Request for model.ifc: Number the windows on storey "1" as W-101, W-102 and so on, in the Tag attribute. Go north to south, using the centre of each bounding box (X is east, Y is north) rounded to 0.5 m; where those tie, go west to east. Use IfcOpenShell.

First a look at what the model holds.

```python
import ifcopenshell
import ifcopenshell.util.element
import ifcopenshell.util.placement

model = ifcopenshell.open("model.ifc")
print(model.schema)
storey = next(s for s in model.by_type("IfcBuildingStorey") if s.Name == "1")
windows = [e for e in ifcopenshell.util.element.get_decomposition(storey) if e.is_a("IfcWindow")]
for e in sorted(windows, key=lambda e: e.id()):
    origin = ifcopenshell.util.placement.get_local_placement(e.ObjectPlacement)[:3, 3]
    print(e.id(), e.Tag, e.Name, origin.round(2) + 0.0, sep=" | ")
```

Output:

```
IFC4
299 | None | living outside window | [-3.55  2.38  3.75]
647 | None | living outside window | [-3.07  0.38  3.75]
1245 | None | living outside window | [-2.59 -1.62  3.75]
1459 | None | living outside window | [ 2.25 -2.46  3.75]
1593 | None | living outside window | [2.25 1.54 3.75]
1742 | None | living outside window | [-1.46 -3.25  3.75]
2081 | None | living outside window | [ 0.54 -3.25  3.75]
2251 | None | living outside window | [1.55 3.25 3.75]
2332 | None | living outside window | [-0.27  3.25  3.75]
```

```python
import ifcopenshell
import ifcopenshell.geom
import ifcopenshell.util.element
import ifcopenshell.util.shape

model = ifcopenshell.open("model.ifc")
settings = ifcopenshell.geom.settings()
settings.set("use-world-coords", True)


def centre(element):
    shape = ifcopenshell.geom.create_shape(settings, element)
    return ifcopenshell.util.shape.get_bbox_centroid(shape.geometry)


storey = next(s for s in model.by_type("IfcBuildingStorey") if s.Name == "1")
windows = [e for e in ifcopenshell.util.element.get_decomposition(storey) if e.is_a("IfcWindow")]

# Insertion points can sit at a corner or the storey origin, so sort by the geometry (in metres).
centres = {e: centre(e) for e in windows}
windows.sort(key=lambda e: (-round(centres[e][1] / 0.5), centres[e][0]))

for i, e in enumerate(windows, start=1):
    number = f"W-1{i:02d}"
    e.Tag = number
    print(e.id(), number)

model.write("model_rev.ifc")
```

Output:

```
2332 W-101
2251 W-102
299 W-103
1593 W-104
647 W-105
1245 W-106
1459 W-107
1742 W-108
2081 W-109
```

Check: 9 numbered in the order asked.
